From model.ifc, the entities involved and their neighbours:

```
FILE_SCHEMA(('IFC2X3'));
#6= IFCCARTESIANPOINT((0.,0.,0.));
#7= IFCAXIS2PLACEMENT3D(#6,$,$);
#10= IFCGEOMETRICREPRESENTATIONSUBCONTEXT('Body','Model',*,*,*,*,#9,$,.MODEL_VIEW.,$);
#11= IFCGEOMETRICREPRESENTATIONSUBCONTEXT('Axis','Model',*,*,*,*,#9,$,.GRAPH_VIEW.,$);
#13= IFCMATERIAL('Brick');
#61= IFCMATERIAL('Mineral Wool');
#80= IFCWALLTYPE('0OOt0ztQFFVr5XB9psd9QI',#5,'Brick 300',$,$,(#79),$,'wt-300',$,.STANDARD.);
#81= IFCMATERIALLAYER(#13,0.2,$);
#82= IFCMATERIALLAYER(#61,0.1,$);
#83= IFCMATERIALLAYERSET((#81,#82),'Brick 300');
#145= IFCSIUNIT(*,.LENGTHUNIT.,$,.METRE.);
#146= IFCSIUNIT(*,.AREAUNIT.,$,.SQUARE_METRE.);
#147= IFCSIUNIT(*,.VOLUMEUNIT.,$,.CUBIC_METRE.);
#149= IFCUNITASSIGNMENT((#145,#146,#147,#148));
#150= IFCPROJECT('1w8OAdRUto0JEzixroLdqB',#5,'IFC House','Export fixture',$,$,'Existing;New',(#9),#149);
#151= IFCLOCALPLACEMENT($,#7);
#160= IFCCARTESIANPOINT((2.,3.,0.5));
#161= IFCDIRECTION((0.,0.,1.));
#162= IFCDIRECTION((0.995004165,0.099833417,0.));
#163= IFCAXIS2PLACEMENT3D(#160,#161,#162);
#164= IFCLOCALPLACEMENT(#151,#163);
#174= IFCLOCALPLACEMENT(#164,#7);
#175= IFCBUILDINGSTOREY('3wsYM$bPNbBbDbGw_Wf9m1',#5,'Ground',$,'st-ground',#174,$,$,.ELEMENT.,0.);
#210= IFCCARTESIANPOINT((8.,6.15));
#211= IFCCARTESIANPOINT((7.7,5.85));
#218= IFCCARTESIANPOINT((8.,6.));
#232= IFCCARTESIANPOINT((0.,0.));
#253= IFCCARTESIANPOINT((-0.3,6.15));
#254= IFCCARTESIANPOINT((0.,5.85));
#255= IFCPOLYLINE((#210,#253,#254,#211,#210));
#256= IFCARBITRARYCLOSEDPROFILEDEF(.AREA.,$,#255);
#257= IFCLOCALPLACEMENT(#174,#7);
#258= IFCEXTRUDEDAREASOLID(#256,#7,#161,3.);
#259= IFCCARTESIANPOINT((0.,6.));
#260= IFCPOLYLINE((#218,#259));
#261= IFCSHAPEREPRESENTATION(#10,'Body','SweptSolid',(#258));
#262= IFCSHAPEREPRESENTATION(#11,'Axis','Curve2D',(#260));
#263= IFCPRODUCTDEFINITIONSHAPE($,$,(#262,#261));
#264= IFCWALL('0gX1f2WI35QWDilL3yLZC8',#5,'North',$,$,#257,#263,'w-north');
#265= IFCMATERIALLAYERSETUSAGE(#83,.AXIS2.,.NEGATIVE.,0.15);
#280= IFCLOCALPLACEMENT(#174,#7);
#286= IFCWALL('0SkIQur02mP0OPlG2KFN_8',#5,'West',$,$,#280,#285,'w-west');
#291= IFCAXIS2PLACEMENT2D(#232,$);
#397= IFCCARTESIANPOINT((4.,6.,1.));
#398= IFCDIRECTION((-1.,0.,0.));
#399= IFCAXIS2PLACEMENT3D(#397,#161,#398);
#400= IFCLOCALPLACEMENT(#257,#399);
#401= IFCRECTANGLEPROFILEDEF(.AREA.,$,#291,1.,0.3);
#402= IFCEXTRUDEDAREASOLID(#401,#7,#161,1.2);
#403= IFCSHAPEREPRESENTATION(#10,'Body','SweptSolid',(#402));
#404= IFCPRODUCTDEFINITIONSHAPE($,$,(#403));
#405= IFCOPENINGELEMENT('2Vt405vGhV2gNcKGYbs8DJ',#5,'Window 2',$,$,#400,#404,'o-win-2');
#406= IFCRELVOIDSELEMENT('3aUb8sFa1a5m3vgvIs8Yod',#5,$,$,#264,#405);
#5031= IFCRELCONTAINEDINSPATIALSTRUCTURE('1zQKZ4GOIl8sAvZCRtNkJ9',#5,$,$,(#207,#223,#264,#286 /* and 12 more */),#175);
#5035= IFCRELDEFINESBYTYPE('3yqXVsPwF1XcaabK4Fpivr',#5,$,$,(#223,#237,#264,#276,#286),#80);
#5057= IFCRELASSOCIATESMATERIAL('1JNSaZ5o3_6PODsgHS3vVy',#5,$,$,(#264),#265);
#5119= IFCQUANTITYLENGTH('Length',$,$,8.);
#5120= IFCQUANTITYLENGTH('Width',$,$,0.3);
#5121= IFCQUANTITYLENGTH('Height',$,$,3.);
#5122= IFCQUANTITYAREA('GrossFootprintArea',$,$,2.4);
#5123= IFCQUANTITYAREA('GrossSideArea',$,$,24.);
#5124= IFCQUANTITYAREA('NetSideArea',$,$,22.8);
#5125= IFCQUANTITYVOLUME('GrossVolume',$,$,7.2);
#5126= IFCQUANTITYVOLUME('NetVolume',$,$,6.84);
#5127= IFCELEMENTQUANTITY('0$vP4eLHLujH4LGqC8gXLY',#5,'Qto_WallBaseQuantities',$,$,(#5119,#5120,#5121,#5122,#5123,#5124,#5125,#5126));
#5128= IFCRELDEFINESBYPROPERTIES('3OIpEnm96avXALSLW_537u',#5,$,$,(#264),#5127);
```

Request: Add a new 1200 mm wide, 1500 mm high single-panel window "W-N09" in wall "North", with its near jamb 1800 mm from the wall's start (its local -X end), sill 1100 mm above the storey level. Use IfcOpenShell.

```python
import numpy as np
import ifcopenshell
import ifcopenshell.api.feature
import ifcopenshell.api.geometry
import ifcopenshell.api.pset
import ifcopenshell.api.root
import ifcopenshell.api.spatial
import ifcopenshell.api.type
import ifcopenshell.geom
import ifcopenshell.util.element
import ifcopenshell.util.placement
import ifcopenshell.util.representation
import ifcopenshell.util.shape
import ifcopenshell.util.unit

model = ifcopenshell.open("model.ifc")
unit_scale = ifcopenshell.util.unit.calculate_unit_scale(model)
area_scale = ifcopenshell.util.unit.calculate_unit_scale(model, "AREAUNIT")
volume_scale = ifcopenshell.util.unit.calculate_unit_scale(model, "VOLUMEUNIT")
settings = ifcopenshell.geom.settings()


def volume(element):
    """Net volume in cubic metres, openings subtracted."""
    shape = ifcopenshell.geom.create_shape(settings, element)
    return ifcopenshell.util.shape.get_volume(shape.geometry)


wall = model.by_guid("0gX1f2WI35QWDilL3yLZC8")
storey = ifcopenshell.util.element.get_container(wall, ifc_class="IfcBuildingStorey")
context = ifcopenshell.util.representation.get_context(model, "Model", "Body", "MODEL_VIEW")
before = volume(wall)

width, height, from_end, sill = 1.2, 1.5, 1.8, 1.1  # metres

# The wall runs along its own X axis, and the end named is its -X end.
wall_shape = ifcopenshell.geom.create_shape(settings, wall)
x, y, z = ifcopenshell.util.shape.get_vertices(wall_shape.geometry).T
start = x.min() + from_end
face, thickness = float(y.min()), float(y.max() - y.min())
wall_matrix = ifcopenshell.util.placement.get_local_placement(wall.ObjectPlacement)
level = ifcopenshell.util.placement.get_local_placement(storey.ObjectPlacement)[2, 3]


def in_wall(x, y):
    """Placement at x, y metres in the wall's axes, at sill height."""
    matrix = wall_matrix.copy()
    matrix[:, 3] = wall_matrix @ np.array([x / unit_scale, y / unit_scale, 0.0, 1.0])
    matrix[2, 3] = level + sill / unit_scale
    return matrix


# Opening: a box that overshoots both wall faces by 50 mm.
opening = ifcopenshell.api.root.create_entity(model, ifc_class="IfcOpeningElement")
box = ifcopenshell.api.geometry.add_wall_representation(
    model, context=context, length=width, height=height, thickness=thickness + 0.1
)
ifcopenshell.api.geometry.assign_representation(model, product=opening, representation=box)
ifcopenshell.api.geometry.edit_object_placement(model, product=opening, matrix=in_wall(start, face - 0.05), is_si=False)
ifcopenshell.api.feature.add_feature(model, feature=opening, element=wall)

window = ifcopenshell.api.root.create_entity(model, ifc_class="IfcWindow", name="W-N09")
window.OverallWidth, window.OverallHeight = width / unit_scale, height / unit_scale
body = ifcopenshell.api.geometry.add_window_representation(
    model,
    context=context,
    overall_width=window.OverallWidth,
    overall_height=window.OverallHeight,
    partition_type="SINGLE_PANEL",
)
ifcopenshell.api.geometry.assign_representation(model, product=window, representation=body)
ifcopenshell.api.spatial.assign_container(model, products=[window], relating_structure=storey)
fills = ifcopenshell.api.feature.add_filling(model, opening=opening, element=window)
fills.OwnerHistory = window.OwnerHistory  # required in IFC2X3

# IFC2X3 keeps the operation on the window style.
style = ifcopenshell.api.root.create_entity(model, ifc_class="IfcWindowStyle", name="W-N09")
style.OperationType, style.ConstructionType = "SINGLE_PANEL", "NOTDEFINED"
style.ParameterTakesPrecedence = style.Sizeable = False
ifcopenshell.api.type.assign_type(model, related_objects=[window], relating_type=style)

# Centre the window in the wall's thickness.
ifcopenshell.api.geometry.edit_object_placement(model, product=window, matrix=in_wall(start, face), is_si=False)
window_shape = ifcopenshell.geom.create_shape(settings, window)
depth = ifcopenshell.util.shape.get_vertices(window_shape.geometry)[:, 1]
offset = face + thickness / 2 - (depth.min() + depth.max()) / 2
ifcopenshell.api.geometry.edit_object_placement(model, product=window, matrix=in_wall(start, offset), is_si=False)

after = volume(wall)

# Update the wall's stored quantities.
qto = model.by_id(ifcopenshell.util.element.get_pset(wall, "Qto_WallBaseQuantities", should_inherit=False)["id"])
ifcopenshell.api.pset.edit_qto(model, qto=qto, properties={
    "NetSideArea": after / thickness / area_scale,
    "NetVolume": after / volume_scale,
})

print(f"wall volume {before:.3f} -> {after:.3f} m3")

model.write("model_v2.ifc")
```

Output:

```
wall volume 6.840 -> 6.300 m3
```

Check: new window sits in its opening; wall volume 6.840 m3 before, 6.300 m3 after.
